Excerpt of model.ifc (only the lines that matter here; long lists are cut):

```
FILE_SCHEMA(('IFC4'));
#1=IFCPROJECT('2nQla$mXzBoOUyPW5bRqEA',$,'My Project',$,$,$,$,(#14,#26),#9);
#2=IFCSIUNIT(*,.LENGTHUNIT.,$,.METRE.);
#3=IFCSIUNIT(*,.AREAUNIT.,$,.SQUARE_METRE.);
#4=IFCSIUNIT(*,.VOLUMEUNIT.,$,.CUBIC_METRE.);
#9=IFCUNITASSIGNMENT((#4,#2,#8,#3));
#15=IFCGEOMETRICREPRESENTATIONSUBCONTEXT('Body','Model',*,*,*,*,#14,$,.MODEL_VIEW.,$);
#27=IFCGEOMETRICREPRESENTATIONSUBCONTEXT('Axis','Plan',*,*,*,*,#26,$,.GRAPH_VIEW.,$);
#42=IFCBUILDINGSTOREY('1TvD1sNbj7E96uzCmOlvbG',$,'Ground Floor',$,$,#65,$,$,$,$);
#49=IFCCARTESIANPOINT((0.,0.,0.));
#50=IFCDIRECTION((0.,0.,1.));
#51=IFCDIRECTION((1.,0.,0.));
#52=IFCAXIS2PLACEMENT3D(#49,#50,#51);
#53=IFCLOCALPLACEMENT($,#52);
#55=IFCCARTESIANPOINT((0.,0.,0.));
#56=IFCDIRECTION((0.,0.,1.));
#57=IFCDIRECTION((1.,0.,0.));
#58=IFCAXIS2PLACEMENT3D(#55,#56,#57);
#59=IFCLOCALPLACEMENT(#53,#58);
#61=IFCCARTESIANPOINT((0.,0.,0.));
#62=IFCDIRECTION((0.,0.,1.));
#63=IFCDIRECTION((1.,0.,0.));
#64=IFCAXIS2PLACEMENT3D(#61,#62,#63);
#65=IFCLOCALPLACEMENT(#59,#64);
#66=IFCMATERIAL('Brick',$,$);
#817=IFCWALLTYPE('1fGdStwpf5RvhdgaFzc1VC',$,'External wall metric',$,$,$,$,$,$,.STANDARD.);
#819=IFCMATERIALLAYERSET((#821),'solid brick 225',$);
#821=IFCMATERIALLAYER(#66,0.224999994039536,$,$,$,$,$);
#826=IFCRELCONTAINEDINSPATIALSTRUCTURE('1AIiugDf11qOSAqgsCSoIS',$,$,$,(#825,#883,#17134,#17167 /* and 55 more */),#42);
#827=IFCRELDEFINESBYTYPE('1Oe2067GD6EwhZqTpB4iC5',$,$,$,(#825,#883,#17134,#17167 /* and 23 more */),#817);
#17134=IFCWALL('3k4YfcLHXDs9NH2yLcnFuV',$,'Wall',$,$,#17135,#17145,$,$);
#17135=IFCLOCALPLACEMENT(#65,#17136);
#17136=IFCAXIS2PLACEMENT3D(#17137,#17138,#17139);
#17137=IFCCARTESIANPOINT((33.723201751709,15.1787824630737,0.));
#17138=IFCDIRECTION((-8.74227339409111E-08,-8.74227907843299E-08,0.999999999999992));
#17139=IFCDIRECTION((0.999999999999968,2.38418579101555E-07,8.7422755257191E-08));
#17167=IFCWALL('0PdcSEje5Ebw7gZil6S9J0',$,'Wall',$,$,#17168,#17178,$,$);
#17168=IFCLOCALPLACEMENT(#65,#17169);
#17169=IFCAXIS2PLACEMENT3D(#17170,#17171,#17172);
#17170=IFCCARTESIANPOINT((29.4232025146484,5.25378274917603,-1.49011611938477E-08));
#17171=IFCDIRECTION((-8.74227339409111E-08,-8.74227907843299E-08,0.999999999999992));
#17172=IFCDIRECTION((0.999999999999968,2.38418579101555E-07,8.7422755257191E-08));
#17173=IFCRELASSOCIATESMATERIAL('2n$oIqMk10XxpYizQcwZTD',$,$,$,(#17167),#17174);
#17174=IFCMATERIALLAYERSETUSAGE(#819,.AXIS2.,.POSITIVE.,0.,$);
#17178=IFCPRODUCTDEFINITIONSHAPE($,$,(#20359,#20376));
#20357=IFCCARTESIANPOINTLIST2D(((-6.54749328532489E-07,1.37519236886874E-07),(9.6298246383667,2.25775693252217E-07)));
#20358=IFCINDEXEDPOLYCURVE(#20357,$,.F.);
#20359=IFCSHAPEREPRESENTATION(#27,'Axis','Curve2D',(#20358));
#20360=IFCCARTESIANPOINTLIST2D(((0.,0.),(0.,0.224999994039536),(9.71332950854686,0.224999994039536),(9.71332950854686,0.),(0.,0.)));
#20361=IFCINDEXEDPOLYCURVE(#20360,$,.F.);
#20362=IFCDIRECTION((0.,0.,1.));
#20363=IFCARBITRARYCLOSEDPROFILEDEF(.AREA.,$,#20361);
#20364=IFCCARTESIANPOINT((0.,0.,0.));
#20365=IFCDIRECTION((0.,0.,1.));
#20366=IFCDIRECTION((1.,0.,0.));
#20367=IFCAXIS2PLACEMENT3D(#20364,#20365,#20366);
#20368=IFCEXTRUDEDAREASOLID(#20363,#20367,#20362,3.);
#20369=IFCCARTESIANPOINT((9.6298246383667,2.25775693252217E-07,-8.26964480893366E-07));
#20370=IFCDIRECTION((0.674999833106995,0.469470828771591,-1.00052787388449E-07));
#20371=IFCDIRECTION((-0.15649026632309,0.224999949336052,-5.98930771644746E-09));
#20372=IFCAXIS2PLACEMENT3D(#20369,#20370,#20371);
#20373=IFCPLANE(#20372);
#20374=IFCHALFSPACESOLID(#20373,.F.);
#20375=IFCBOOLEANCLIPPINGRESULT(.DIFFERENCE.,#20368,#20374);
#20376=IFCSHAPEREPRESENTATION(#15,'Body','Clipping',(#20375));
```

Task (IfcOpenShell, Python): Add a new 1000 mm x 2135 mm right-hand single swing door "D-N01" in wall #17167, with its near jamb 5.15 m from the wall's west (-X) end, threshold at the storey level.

```python
import numpy as np
import ifcopenshell
import ifcopenshell.api.feature
import ifcopenshell.api.geometry
import ifcopenshell.api.root
import ifcopenshell.api.spatial
import ifcopenshell.geom
import ifcopenshell.util.element
import ifcopenshell.util.placement
import ifcopenshell.util.representation
import ifcopenshell.util.shape
import ifcopenshell.util.unit

model = ifcopenshell.open("model.ifc")
unit_scale = ifcopenshell.util.unit.calculate_unit_scale(model)
settings = ifcopenshell.geom.settings()


def volume(element):
    """Net volume in cubic metres, openings subtracted."""
    shape = ifcopenshell.geom.create_shape(settings, element)
    return ifcopenshell.util.shape.get_volume(shape.geometry)


wall = model.by_guid("0PdcSEje5Ebw7gZil6S9J0")
storey = ifcopenshell.util.element.get_container(wall, ifc_class="IfcBuildingStorey")
context = ifcopenshell.util.representation.get_context(model, "Model", "Body", "MODEL_VIEW")
before = volume(wall)

width, height, from_end, sill = 1, 2.135, 5.15, 0.0  # metres

# The wall runs along its own X axis, and the end named is its -X end.
wall_shape = ifcopenshell.geom.create_shape(settings, wall)
x, y, z = ifcopenshell.util.shape.get_vertices(wall_shape.geometry).T
start = x.min() + from_end
face, thickness = float(y.min()), float(y.max() - y.min())
wall_matrix = ifcopenshell.util.placement.get_local_placement(wall.ObjectPlacement)
level = ifcopenshell.util.placement.get_local_placement(storey.ObjectPlacement)[2, 3]


def in_wall(x, y):
    """Placement at x, y metres in the wall's axes, at sill height."""
    matrix = wall_matrix.copy()
    matrix[:, 3] = wall_matrix @ np.array([x / unit_scale, y / unit_scale, 0.0, 1.0])
    matrix[2, 3] = level + sill / unit_scale
    return matrix


# Opening: a box that overshoots both wall faces by 50 mm.
opening = ifcopenshell.api.root.create_entity(model, ifc_class="IfcOpeningElement", predefined_type="OPENING")
box = ifcopenshell.api.geometry.add_wall_representation(
    model, context=context, length=width, height=height, thickness=thickness + 0.1
)
ifcopenshell.api.geometry.assign_representation(model, product=opening, representation=box)
ifcopenshell.api.geometry.edit_object_placement(model, product=opening, matrix=in_wall(start, face - 0.05), is_si=False)
ifcopenshell.api.feature.add_feature(model, feature=opening, element=wall)

door = ifcopenshell.api.root.create_entity(model, ifc_class="IfcDoor", name="D-N01", predefined_type="DOOR")
door.OverallWidth, door.OverallHeight = width / unit_scale, height / unit_scale
door.OperationType = "SINGLE_SWING_RIGHT"
body = ifcopenshell.api.geometry.add_door_representation(
    model,
    context=context,
    overall_width=door.OverallWidth,
    overall_height=door.OverallHeight,
    operation_type="SINGLE_SWING_RIGHT",
    lining_properties={"LiningDepth": thickness / unit_scale, "ThresholdDepth": thickness / unit_scale},
)
ifcopenshell.api.geometry.assign_representation(model, product=door, representation=body)
ifcopenshell.api.spatial.assign_container(model, products=[door], relating_structure=storey)
ifcopenshell.api.feature.add_filling(model, opening=opening, element=door)

# The lining spans the wall, so the door starts at the wall face.
ifcopenshell.api.geometry.edit_object_placement(model, product=door, matrix=in_wall(start, face), is_si=False)

after = volume(wall)

print(f"wall volume {before:.3f} -> {after:.3f} m3")

model.write("model_updated.ifc")
```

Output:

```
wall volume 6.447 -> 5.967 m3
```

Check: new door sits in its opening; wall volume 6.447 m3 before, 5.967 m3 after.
